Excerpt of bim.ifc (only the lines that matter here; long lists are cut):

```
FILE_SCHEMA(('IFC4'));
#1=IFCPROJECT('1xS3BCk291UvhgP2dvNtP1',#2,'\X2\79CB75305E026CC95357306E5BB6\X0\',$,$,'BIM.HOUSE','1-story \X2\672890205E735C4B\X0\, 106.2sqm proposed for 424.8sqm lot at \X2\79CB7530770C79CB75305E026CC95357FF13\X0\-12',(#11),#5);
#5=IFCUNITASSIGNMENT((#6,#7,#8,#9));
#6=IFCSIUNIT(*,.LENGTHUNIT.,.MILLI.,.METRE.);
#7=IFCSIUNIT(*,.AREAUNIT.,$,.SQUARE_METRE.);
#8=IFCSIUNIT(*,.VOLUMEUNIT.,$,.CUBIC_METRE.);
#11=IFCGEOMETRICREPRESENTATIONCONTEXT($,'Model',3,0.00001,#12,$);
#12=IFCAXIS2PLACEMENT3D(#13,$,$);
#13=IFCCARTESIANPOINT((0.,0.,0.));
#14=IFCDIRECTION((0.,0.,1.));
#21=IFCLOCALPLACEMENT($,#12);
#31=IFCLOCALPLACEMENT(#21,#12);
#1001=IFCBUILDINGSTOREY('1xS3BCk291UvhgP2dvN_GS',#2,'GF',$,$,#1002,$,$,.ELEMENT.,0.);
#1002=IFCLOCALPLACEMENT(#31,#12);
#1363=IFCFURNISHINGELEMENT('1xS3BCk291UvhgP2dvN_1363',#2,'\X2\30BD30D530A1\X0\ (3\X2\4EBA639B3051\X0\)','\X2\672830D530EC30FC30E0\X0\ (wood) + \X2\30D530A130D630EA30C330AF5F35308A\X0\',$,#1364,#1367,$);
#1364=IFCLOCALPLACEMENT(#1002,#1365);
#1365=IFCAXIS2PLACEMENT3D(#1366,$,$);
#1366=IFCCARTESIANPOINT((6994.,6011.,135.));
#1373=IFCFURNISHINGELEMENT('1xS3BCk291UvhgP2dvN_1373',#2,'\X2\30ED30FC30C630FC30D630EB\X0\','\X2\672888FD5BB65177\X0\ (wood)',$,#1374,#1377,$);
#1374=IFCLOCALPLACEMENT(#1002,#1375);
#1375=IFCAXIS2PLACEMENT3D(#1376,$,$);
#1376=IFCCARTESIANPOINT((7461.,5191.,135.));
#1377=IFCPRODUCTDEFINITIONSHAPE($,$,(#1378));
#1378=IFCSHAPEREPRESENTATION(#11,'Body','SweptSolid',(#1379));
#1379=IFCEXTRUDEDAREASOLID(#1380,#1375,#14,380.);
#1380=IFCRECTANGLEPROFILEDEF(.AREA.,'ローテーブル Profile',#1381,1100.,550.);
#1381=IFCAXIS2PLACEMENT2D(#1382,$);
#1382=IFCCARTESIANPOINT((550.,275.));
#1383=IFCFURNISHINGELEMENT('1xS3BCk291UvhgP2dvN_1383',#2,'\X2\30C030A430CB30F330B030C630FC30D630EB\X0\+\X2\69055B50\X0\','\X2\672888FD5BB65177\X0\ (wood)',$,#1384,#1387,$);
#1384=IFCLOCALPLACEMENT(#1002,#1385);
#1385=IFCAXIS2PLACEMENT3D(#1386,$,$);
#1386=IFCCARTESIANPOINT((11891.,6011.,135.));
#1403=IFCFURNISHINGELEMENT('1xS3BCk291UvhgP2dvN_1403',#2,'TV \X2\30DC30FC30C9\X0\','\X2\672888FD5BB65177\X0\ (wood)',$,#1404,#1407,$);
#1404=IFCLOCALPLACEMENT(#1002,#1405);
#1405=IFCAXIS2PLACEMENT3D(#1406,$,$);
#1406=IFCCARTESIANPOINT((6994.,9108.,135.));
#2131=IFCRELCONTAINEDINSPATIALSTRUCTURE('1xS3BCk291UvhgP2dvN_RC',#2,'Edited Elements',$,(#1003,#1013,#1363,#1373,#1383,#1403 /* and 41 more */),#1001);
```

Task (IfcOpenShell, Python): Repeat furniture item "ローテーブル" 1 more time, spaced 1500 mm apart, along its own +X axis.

```python
import ifcopenshell
import ifcopenshell.api.geometry
import ifcopenshell.api.root
import ifcopenshell.util.element
import ifcopenshell.util.placement
import ifcopenshell.util.unit

model = ifcopenshell.open("bim.ifc")
unit_scale = ifcopenshell.util.unit.calculate_unit_scale(model)


def reuse_history(source, copy):
    """copy_class also copies each property set's owner history, people and application; keep the originals."""
    for rel in copy.IsDefinedBy:
        if rel.is_a("IfcRelDefinesByProperties") and (history := rel.RelatingPropertyDefinition.OwnerHistory):
            rel.RelatingPropertyDefinition.OwnerHistory = source.OwnerHistory
            ifcopenshell.util.element.remove_deep2(model, history)


source = model.by_id(1373)
base = ifcopenshell.util.placement.get_local_placement(source.ObjectPlacement)
step = base[:3, 0] * 1.5 / unit_scale

for i in range(1, 2):
    copy = ifcopenshell.api.root.copy_class(model, product=source)
    copy.Representation = ifcopenshell.util.element.copy_deep(
        model, source.Representation, exclude=["IfcGeometricRepresentationContext", "IfcRepresentationMap"]
    )
    reuse_history(source, copy)
    matrix = base.copy()
    matrix[:3, 3] += i * step
    print("added at", matrix[:3, 3].round(3) + 0.0)
    ifcopenshell.api.geometry.edit_object_placement(model, product=copy, matrix=matrix, is_si=False)

model.write("bim_v2.ifc")
```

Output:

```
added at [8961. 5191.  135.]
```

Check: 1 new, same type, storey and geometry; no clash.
